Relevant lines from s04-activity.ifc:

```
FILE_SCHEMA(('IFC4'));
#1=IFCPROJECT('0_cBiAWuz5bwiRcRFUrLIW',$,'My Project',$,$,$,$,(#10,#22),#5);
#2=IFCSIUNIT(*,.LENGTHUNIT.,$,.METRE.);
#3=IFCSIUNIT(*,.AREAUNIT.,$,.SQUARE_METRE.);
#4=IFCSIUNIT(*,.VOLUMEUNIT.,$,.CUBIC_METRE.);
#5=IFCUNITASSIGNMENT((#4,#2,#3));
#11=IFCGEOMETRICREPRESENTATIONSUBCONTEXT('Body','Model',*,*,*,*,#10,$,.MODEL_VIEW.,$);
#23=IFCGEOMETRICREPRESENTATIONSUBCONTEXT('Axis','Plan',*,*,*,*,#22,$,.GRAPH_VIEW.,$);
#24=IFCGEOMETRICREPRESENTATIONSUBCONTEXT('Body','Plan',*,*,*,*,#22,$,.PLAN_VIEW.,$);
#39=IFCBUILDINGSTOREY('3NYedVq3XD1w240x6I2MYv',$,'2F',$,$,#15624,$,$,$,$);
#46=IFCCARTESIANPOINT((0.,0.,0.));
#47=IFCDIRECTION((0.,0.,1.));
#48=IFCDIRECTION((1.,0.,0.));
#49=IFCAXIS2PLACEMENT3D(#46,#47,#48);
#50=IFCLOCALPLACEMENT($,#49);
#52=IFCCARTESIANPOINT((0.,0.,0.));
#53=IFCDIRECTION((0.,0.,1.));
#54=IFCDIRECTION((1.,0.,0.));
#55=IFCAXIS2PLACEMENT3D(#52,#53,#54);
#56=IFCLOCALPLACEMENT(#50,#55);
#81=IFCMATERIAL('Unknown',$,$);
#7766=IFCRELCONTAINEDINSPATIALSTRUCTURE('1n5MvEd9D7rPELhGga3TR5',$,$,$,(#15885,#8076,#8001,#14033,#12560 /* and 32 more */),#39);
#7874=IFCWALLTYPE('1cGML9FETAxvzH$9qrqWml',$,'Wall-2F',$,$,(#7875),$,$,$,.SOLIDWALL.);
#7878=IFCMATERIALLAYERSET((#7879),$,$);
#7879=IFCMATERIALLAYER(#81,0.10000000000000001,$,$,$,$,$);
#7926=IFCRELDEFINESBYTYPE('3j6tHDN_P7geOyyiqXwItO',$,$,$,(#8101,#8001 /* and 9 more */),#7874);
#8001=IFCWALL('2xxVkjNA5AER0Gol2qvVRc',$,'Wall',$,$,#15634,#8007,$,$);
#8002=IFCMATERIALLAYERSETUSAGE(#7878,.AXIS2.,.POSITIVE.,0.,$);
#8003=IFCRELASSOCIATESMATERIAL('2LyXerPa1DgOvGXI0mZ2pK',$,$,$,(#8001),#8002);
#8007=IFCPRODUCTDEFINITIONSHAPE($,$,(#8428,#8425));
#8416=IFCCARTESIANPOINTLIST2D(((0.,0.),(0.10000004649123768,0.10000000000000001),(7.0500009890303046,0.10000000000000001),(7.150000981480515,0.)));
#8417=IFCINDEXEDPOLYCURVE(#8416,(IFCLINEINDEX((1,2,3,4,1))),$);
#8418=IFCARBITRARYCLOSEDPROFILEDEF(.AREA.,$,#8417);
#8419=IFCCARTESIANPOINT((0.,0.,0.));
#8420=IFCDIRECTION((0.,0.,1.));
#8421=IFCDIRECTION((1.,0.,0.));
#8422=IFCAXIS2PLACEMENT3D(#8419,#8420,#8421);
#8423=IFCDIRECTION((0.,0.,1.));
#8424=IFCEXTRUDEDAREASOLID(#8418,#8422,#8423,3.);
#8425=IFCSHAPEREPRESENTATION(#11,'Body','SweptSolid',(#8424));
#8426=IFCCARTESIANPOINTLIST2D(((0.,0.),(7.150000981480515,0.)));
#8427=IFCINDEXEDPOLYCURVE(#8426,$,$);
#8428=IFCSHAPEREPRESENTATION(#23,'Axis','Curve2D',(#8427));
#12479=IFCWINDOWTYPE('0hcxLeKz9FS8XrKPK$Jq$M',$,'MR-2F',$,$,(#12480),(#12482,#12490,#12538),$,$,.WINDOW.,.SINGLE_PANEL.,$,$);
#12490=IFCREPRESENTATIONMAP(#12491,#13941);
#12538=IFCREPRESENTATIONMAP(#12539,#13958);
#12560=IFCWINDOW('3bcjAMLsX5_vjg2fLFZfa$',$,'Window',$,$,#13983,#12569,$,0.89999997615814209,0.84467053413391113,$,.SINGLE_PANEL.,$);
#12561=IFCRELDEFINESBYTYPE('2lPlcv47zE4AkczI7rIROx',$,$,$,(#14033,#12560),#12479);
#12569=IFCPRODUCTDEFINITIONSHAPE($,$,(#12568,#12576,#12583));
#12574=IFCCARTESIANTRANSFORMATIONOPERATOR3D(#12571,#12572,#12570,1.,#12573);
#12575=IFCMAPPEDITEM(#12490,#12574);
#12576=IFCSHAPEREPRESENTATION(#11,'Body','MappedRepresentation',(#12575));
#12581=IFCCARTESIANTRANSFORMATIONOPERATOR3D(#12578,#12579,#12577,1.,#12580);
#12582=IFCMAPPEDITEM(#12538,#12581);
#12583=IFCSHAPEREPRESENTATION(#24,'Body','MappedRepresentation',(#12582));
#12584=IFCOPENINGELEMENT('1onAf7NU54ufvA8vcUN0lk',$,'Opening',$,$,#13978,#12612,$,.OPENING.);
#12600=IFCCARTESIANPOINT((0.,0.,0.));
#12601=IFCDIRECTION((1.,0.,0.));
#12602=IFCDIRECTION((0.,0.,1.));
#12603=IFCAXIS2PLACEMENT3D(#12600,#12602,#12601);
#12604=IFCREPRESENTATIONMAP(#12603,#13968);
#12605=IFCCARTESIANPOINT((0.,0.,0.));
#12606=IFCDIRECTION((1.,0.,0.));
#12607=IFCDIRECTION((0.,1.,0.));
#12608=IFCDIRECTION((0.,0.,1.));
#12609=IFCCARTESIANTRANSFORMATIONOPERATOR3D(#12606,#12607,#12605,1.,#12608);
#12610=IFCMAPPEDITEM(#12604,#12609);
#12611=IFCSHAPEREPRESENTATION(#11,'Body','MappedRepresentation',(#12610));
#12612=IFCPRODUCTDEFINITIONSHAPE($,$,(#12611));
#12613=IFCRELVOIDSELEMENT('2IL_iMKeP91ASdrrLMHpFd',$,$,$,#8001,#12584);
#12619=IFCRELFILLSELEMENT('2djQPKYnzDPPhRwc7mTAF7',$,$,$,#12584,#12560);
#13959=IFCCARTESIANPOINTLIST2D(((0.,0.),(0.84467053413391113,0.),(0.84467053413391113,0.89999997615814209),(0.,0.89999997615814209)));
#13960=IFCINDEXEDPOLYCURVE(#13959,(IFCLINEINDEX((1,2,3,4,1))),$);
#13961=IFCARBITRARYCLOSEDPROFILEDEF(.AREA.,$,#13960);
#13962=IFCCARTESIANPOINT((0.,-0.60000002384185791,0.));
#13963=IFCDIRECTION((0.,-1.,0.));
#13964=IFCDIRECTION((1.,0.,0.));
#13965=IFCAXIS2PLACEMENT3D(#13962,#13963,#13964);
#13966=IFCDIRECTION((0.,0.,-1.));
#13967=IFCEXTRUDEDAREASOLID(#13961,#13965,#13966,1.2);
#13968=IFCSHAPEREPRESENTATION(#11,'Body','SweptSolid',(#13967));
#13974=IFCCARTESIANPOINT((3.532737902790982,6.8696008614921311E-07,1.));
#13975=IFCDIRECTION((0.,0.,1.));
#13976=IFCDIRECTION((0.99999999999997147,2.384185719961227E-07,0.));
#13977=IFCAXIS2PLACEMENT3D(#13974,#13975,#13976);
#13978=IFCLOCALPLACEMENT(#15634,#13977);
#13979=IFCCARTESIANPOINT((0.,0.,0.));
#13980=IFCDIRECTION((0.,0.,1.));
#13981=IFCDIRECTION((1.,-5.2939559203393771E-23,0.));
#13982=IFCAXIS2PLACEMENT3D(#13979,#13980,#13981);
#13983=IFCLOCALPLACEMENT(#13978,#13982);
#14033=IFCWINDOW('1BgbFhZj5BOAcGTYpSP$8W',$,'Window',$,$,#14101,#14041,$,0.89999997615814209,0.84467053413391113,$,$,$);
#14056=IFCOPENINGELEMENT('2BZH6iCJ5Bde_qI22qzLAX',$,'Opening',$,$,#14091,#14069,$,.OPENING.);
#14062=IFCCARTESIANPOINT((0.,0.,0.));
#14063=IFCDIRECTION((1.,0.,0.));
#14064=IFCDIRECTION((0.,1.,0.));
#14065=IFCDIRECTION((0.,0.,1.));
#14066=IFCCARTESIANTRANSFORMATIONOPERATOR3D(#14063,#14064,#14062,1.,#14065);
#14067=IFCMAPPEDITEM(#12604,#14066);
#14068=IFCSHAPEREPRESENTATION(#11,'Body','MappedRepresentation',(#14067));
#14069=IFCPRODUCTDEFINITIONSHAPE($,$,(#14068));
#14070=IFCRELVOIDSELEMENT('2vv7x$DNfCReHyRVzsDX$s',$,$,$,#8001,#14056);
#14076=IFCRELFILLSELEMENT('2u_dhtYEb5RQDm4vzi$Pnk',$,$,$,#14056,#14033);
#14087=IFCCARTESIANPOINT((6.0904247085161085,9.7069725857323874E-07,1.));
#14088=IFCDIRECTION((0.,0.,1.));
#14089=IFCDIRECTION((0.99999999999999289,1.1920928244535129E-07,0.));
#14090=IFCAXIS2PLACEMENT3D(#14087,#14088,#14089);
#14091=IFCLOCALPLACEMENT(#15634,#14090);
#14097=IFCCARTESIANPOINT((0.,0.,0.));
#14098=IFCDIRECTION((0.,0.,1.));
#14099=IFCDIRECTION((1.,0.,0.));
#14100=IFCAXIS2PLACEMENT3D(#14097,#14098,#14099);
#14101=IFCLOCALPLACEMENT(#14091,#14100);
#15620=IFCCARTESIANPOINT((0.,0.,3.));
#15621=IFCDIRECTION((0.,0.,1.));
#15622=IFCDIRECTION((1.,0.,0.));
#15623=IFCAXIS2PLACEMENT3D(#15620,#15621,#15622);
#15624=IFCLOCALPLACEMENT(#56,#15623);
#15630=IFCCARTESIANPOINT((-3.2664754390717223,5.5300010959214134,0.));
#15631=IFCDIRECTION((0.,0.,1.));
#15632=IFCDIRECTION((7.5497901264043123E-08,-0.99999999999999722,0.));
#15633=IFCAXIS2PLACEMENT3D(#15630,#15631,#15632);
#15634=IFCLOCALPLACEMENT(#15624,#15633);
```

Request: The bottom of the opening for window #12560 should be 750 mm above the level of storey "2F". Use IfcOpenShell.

```python
import numpy as np
import ifcopenshell
import ifcopenshell.api.geometry
import ifcopenshell.geom
import ifcopenshell.util.element
import ifcopenshell.util.placement
import ifcopenshell.util.shape
import ifcopenshell.util.unit

model = ifcopenshell.open("s04-activity.ifc")
unit_scale = ifcopenshell.util.unit.calculate_unit_scale(model)

window = model.by_guid("3bcjAMLsX5_vjg2fLFZfa$")
opening = window.FillsVoids[0].RelatingOpeningElement
storey = ifcopenshell.util.element.get_container(window, ifc_class="IfcBuildingStorey")
level = ifcopenshell.util.placement.get_local_placement(storey.ObjectPlacement)[2, 3]

# The opening's origin need not be at the sill, so measure its lowest point.
shape = ifcopenshell.geom.create_shape(ifcopenshell.geom.settings(), opening)
bottom = ifcopenshell.util.shape.get_shape_bottom_elevation(shape, shape.geometry) / unit_scale
dz = level + 0.75 - bottom

shift = np.array([0.0, 0.0, dz])
# The window is placed relative to its opening, so it follows when the opening moves.
matrix = ifcopenshell.util.placement.get_local_placement(opening.ObjectPlacement)
matrix[:3, 3] += shift
ifcopenshell.api.geometry.edit_object_placement(
    model, product=opening, matrix=matrix, is_si=False, should_transform_children=True
)

print(f"moved by {dz * unit_scale:+.3f} m")

model.write("s04-activity_edited.ifc")
```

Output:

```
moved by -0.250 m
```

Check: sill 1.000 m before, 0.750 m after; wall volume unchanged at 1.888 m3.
